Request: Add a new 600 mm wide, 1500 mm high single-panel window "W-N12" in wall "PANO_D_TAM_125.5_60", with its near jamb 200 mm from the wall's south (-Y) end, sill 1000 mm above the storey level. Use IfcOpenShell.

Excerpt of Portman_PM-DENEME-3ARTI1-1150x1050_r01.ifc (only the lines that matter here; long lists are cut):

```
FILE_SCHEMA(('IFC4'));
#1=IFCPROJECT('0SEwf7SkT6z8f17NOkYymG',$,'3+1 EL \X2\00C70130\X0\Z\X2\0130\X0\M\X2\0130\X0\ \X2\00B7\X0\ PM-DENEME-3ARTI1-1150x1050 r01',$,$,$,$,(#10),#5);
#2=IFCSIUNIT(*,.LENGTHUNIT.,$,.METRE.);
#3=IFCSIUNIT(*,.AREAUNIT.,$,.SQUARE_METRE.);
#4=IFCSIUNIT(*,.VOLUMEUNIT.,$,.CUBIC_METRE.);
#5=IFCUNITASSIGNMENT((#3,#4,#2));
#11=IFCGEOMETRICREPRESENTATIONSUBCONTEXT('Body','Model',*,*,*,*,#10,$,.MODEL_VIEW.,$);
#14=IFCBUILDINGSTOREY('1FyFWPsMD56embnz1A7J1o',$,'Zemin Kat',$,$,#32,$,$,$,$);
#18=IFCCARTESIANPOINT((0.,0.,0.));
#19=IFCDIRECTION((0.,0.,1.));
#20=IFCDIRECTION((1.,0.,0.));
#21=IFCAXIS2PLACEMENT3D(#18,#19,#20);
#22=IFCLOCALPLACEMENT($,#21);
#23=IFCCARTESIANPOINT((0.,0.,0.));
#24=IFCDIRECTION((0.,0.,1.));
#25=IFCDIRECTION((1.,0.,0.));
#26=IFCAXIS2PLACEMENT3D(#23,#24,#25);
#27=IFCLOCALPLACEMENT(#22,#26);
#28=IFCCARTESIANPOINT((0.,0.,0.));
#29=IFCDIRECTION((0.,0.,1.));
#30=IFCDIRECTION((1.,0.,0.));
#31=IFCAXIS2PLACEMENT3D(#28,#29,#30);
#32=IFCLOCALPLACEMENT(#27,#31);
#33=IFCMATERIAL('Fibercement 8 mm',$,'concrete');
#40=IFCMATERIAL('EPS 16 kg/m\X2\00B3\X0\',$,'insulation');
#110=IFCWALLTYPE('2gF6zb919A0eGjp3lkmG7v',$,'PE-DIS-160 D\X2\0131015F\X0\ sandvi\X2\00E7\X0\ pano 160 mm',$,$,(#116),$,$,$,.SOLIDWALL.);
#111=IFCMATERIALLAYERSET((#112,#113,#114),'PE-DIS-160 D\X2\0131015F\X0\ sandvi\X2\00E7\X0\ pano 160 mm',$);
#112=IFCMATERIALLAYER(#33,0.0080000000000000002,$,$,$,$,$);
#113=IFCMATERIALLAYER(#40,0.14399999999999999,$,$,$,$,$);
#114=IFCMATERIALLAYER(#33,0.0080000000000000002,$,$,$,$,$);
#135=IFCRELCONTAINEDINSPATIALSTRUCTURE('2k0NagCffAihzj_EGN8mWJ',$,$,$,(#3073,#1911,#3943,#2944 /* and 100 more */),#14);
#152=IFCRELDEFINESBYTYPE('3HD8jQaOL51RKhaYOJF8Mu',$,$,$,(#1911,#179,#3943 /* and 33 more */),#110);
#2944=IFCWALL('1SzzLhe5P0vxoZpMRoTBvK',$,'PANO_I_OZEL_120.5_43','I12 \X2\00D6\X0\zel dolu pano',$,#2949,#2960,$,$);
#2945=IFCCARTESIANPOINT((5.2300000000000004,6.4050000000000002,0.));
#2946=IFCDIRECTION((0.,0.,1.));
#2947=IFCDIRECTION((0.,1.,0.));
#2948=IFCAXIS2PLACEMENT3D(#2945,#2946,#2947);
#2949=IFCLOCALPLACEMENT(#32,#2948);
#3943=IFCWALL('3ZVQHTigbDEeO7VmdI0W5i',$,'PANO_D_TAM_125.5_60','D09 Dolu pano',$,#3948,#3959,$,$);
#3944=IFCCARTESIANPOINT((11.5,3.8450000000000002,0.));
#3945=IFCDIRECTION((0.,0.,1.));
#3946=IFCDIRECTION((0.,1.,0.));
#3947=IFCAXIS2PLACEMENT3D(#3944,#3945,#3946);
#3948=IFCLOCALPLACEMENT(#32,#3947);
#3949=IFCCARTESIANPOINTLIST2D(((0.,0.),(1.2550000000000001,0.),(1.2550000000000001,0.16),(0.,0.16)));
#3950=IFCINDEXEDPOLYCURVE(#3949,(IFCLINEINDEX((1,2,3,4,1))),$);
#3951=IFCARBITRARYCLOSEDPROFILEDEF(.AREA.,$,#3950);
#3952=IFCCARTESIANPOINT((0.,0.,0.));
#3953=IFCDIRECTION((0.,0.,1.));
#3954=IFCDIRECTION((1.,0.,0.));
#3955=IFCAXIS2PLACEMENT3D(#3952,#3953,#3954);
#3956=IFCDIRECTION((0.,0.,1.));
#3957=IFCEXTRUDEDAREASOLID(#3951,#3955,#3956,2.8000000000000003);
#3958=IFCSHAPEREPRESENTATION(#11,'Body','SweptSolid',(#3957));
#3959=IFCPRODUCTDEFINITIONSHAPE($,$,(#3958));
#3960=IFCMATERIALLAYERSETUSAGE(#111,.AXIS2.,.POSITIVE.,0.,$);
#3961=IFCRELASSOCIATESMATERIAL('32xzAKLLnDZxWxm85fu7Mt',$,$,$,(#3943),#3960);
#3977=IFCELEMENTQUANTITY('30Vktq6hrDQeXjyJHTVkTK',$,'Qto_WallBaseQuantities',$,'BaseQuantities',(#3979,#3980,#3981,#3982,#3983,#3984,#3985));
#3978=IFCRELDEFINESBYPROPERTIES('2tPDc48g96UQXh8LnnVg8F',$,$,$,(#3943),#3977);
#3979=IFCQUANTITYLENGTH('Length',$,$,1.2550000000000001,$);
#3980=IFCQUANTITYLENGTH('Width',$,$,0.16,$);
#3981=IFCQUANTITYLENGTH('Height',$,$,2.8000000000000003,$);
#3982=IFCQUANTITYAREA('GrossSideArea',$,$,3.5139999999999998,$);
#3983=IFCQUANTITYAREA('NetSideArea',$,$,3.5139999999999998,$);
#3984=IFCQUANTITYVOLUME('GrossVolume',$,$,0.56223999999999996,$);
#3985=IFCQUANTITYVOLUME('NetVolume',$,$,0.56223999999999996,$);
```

```python
import numpy as np
import ifcopenshell
import ifcopenshell.api.feature
import ifcopenshell.api.geometry
import ifcopenshell.api.pset
import ifcopenshell.api.root
import ifcopenshell.api.spatial
import ifcopenshell.geom
import ifcopenshell.util.element
import ifcopenshell.util.placement
import ifcopenshell.util.representation
import ifcopenshell.util.shape
import ifcopenshell.util.unit

model = ifcopenshell.open("Portman_PM-DENEME-3ARTI1-1150x1050_r01.ifc")
unit_scale = ifcopenshell.util.unit.calculate_unit_scale(model)
area_scale = ifcopenshell.util.unit.calculate_unit_scale(model, "AREAUNIT")
volume_scale = ifcopenshell.util.unit.calculate_unit_scale(model, "VOLUMEUNIT")
settings = ifcopenshell.geom.settings()


def volume(element):
    """Net volume in cubic metres, openings subtracted."""
    shape = ifcopenshell.geom.create_shape(settings, element)
    return ifcopenshell.util.shape.get_volume(shape.geometry)


wall = model.by_guid("3ZVQHTigbDEeO7VmdI0W5i")
storey = ifcopenshell.util.element.get_container(wall, ifc_class="IfcBuildingStorey")
context = ifcopenshell.util.representation.get_context(model, "Model", "Body", "MODEL_VIEW")
before = volume(wall)

width, height, from_end, sill = 0.6, 1.5, 0.2, 1  # metres

# The wall runs along its own X axis, and the end named is its -X end.
wall_shape = ifcopenshell.geom.create_shape(settings, wall)
x, y, z = ifcopenshell.util.shape.get_vertices(wall_shape.geometry).T
start = x.min() + from_end
face, thickness = float(y.min()), float(y.max() - y.min())
wall_matrix = ifcopenshell.util.placement.get_local_placement(wall.ObjectPlacement)
level = ifcopenshell.util.placement.get_local_placement(storey.ObjectPlacement)[2, 3]


def in_wall(x, y):
    """Placement at x, y metres in the wall's axes, at sill height."""
    matrix = wall_matrix.copy()
    matrix[:, 3] = wall_matrix @ np.array([x / unit_scale, y / unit_scale, 0.0, 1.0])
    matrix[2, 3] = level + sill / unit_scale
    return matrix


# Opening: a box that overshoots both wall faces by 50 mm.
opening = ifcopenshell.api.root.create_entity(model, ifc_class="IfcOpeningElement", predefined_type="OPENING")
box = ifcopenshell.api.geometry.add_wall_representation(
    model, context=context, length=width, height=height, thickness=thickness + 0.1
)
ifcopenshell.api.geometry.assign_representation(model, product=opening, representation=box)
ifcopenshell.api.geometry.edit_object_placement(model, product=opening, matrix=in_wall(start, face - 0.05), is_si=False)
ifcopenshell.api.feature.add_feature(model, feature=opening, element=wall)

window = ifcopenshell.api.root.create_entity(model, ifc_class="IfcWindow", name="W-N12", predefined_type="WINDOW")
window.OverallWidth, window.OverallHeight = width / unit_scale, height / unit_scale
window.PartitioningType = "SINGLE_PANEL"
body = ifcopenshell.api.geometry.add_window_representation(
    model,
    context=context,
    overall_width=window.OverallWidth,
    overall_height=window.OverallHeight,
    partition_type="SINGLE_PANEL",
)
ifcopenshell.api.geometry.assign_representation(model, product=window, representation=body)
ifcopenshell.api.spatial.assign_container(model, products=[window], relating_structure=storey)
ifcopenshell.api.feature.add_filling(model, opening=opening, element=window)

# Centre the window in the wall's thickness.
ifcopenshell.api.geometry.edit_object_placement(model, product=window, matrix=in_wall(start, face), is_si=False)
window_shape = ifcopenshell.geom.create_shape(settings, window)
depth = ifcopenshell.util.shape.get_vertices(window_shape.geometry)[:, 1]
offset = face + thickness / 2 - (depth.min() + depth.max()) / 2
ifcopenshell.api.geometry.edit_object_placement(model, product=window, matrix=in_wall(start, offset), is_si=False)

after = volume(wall)

# Update the wall's stored quantities.
qto = model.by_id(ifcopenshell.util.element.get_pset(wall, "Qto_WallBaseQuantities", should_inherit=False)["id"])
ifcopenshell.api.pset.edit_qto(model, qto=qto, properties={
    "NetSideArea": after / thickness / area_scale,
    "NetVolume": after / volume_scale,
})

print(f"wall volume {before:.3f} -> {after:.3f} m3")

model.write("Portman_PM-DENEME-3ARTI1-1150x1050_r01_edited.ifc")
```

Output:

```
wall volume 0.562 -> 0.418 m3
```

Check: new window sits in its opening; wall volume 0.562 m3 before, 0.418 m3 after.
